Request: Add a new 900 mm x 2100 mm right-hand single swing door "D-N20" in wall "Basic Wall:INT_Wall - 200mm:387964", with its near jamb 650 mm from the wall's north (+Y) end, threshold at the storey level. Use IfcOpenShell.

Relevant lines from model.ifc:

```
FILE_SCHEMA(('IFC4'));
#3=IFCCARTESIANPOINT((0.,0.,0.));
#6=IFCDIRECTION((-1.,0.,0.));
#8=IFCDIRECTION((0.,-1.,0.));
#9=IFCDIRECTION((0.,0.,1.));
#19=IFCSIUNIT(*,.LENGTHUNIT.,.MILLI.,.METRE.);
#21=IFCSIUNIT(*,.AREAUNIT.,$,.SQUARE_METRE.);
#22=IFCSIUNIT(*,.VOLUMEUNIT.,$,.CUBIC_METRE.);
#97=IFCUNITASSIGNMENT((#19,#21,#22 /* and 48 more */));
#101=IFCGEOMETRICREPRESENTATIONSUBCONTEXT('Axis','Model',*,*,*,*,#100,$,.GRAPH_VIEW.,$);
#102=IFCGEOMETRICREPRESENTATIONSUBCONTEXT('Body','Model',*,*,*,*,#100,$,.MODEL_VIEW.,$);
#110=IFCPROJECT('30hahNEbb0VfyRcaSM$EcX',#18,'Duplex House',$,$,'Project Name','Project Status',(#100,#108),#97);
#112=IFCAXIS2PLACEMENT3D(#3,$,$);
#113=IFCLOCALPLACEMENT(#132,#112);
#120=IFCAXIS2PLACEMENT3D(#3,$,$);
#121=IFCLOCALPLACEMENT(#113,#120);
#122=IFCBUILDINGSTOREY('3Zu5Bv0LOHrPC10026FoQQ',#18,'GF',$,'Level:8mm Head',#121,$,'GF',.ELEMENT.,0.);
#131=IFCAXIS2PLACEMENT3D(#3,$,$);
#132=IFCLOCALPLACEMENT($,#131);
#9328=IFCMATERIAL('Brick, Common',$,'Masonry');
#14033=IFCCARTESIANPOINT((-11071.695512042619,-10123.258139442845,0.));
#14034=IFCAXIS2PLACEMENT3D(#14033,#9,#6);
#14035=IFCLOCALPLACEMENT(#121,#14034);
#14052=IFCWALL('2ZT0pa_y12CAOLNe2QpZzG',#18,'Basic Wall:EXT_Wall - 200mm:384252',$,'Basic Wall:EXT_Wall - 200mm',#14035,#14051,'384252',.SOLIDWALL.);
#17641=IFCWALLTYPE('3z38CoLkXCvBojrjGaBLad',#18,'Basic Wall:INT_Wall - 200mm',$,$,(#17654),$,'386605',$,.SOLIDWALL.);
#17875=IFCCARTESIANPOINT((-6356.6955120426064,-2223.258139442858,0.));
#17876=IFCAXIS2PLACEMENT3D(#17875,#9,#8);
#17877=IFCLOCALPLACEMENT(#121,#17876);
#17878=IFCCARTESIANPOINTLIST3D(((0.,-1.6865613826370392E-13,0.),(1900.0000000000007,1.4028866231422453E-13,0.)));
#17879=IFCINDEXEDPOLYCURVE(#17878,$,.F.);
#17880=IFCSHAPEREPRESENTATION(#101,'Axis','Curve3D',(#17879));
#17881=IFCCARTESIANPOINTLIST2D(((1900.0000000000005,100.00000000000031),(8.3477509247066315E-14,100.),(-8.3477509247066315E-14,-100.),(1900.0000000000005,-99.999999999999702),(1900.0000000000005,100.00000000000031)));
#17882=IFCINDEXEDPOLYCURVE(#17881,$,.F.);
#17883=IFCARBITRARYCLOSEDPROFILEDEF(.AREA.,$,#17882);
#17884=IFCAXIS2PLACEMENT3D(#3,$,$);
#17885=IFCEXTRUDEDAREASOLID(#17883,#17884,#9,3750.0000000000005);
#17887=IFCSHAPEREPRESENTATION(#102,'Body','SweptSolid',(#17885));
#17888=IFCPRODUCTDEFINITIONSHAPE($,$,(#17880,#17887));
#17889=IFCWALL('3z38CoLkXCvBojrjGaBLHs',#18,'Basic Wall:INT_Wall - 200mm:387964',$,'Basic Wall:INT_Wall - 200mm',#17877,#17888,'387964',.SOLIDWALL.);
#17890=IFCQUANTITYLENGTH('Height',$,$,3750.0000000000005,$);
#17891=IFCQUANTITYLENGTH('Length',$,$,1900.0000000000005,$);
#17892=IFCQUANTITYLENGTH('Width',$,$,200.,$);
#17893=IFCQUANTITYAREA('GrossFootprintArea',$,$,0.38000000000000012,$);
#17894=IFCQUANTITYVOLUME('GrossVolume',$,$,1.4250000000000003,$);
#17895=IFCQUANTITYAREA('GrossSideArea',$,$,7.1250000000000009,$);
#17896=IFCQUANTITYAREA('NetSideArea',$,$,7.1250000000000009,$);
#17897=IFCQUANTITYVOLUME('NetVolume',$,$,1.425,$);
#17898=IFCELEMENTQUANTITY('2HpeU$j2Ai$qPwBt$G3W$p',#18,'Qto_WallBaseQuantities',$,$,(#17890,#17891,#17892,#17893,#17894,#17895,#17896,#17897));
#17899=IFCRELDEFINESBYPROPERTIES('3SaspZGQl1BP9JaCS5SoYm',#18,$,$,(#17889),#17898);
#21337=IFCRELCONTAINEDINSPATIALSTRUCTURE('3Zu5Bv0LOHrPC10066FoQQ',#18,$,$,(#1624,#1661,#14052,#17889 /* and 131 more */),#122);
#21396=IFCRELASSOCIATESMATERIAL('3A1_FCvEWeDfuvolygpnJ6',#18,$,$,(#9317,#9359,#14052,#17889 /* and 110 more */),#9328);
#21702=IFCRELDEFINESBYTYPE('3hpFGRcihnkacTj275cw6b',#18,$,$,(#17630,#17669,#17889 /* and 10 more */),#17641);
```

```python
import numpy as np
import ifcopenshell
import ifcopenshell.api.feature
import ifcopenshell.api.geometry
import ifcopenshell.api.pset
import ifcopenshell.api.root
import ifcopenshell.api.spatial
import ifcopenshell.geom
import ifcopenshell.util.element
import ifcopenshell.util.placement
import ifcopenshell.util.representation
import ifcopenshell.util.shape
import ifcopenshell.util.unit

model = ifcopenshell.open("model.ifc")
unit_scale = ifcopenshell.util.unit.calculate_unit_scale(model)
area_scale = ifcopenshell.util.unit.calculate_unit_scale(model, "AREAUNIT")
volume_scale = ifcopenshell.util.unit.calculate_unit_scale(model, "VOLUMEUNIT")
settings = ifcopenshell.geom.settings()


def volume(element):
    """Net volume in cubic metres, openings subtracted."""
    shape = ifcopenshell.geom.create_shape(settings, element)
    return ifcopenshell.util.shape.get_volume(shape.geometry)


wall = model.by_guid("3z38CoLkXCvBojrjGaBLHs")
storey = ifcopenshell.util.element.get_container(wall, ifc_class="IfcBuildingStorey")
context = ifcopenshell.util.representation.get_context(model, "Model", "Body", "MODEL_VIEW")
before = volume(wall)

width, height, from_end, sill = 0.9, 2.1, 0.65, 0.0  # metres

# The wall runs along its own X axis, and the end named is its -X end.
wall_shape = ifcopenshell.geom.create_shape(settings, wall)
x, y, z = ifcopenshell.util.shape.get_vertices(wall_shape.geometry).T
start = x.min() + from_end
face, thickness = float(y.min()), float(y.max() - y.min())
wall_matrix = ifcopenshell.util.placement.get_local_placement(wall.ObjectPlacement)
level = ifcopenshell.util.placement.get_local_placement(storey.ObjectPlacement)[2, 3]


def in_wall(x, y):
    """Placement at x, y metres in the wall's axes, at sill height."""
    matrix = wall_matrix.copy()
    matrix[:, 3] = wall_matrix @ np.array([x / unit_scale, y / unit_scale, 0.0, 1.0])
    matrix[2, 3] = level + sill / unit_scale
    return matrix


# Opening: a box that overshoots both wall faces by 50 mm.
opening = ifcopenshell.api.root.create_entity(model, ifc_class="IfcOpeningElement", predefined_type="OPENING")
box = ifcopenshell.api.geometry.add_wall_representation(
    model, context=context, length=width, height=height, thickness=thickness + 0.1
)
ifcopenshell.api.geometry.assign_representation(model, product=opening, representation=box)
ifcopenshell.api.geometry.edit_object_placement(model, product=opening, matrix=in_wall(start, face - 0.05), is_si=False)
ifcopenshell.api.feature.add_feature(model, feature=opening, element=wall)

door = ifcopenshell.api.root.create_entity(model, ifc_class="IfcDoor", name="D-N20", predefined_type="DOOR")
door.OverallWidth, door.OverallHeight = width / unit_scale, height / unit_scale
door.OperationType = "SINGLE_SWING_RIGHT"
body = ifcopenshell.api.geometry.add_door_representation(
    model,
    context=context,
    overall_width=door.OverallWidth,
    overall_height=door.OverallHeight,
    operation_type="SINGLE_SWING_RIGHT",
    lining_properties={"LiningDepth": thickness / unit_scale, "ThresholdDepth": thickness / unit_scale},
)
ifcopenshell.api.geometry.assign_representation(model, product=door, representation=body)
ifcopenshell.api.spatial.assign_container(model, products=[door], relating_structure=storey)
ifcopenshell.api.feature.add_filling(model, opening=opening, element=door)

# The lining spans the wall, so the door starts at the wall face.
ifcopenshell.api.geometry.edit_object_placement(model, product=door, matrix=in_wall(start, face), is_si=False)

after = volume(wall)

# Update the wall's stored quantities.
qto = model.by_id(ifcopenshell.util.element.get_pset(wall, "Qto_WallBaseQuantities", should_inherit=False)["id"])
ifcopenshell.api.pset.edit_qto(model, qto=qto, properties={
    "NetSideArea": after / thickness / area_scale,
    "NetVolume": after / volume_scale,
})

print(f"wall volume {before:.3f} -> {after:.3f} m3")

model.write("model_edited.ifc")
```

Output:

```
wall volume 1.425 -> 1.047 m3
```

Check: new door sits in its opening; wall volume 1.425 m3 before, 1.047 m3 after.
